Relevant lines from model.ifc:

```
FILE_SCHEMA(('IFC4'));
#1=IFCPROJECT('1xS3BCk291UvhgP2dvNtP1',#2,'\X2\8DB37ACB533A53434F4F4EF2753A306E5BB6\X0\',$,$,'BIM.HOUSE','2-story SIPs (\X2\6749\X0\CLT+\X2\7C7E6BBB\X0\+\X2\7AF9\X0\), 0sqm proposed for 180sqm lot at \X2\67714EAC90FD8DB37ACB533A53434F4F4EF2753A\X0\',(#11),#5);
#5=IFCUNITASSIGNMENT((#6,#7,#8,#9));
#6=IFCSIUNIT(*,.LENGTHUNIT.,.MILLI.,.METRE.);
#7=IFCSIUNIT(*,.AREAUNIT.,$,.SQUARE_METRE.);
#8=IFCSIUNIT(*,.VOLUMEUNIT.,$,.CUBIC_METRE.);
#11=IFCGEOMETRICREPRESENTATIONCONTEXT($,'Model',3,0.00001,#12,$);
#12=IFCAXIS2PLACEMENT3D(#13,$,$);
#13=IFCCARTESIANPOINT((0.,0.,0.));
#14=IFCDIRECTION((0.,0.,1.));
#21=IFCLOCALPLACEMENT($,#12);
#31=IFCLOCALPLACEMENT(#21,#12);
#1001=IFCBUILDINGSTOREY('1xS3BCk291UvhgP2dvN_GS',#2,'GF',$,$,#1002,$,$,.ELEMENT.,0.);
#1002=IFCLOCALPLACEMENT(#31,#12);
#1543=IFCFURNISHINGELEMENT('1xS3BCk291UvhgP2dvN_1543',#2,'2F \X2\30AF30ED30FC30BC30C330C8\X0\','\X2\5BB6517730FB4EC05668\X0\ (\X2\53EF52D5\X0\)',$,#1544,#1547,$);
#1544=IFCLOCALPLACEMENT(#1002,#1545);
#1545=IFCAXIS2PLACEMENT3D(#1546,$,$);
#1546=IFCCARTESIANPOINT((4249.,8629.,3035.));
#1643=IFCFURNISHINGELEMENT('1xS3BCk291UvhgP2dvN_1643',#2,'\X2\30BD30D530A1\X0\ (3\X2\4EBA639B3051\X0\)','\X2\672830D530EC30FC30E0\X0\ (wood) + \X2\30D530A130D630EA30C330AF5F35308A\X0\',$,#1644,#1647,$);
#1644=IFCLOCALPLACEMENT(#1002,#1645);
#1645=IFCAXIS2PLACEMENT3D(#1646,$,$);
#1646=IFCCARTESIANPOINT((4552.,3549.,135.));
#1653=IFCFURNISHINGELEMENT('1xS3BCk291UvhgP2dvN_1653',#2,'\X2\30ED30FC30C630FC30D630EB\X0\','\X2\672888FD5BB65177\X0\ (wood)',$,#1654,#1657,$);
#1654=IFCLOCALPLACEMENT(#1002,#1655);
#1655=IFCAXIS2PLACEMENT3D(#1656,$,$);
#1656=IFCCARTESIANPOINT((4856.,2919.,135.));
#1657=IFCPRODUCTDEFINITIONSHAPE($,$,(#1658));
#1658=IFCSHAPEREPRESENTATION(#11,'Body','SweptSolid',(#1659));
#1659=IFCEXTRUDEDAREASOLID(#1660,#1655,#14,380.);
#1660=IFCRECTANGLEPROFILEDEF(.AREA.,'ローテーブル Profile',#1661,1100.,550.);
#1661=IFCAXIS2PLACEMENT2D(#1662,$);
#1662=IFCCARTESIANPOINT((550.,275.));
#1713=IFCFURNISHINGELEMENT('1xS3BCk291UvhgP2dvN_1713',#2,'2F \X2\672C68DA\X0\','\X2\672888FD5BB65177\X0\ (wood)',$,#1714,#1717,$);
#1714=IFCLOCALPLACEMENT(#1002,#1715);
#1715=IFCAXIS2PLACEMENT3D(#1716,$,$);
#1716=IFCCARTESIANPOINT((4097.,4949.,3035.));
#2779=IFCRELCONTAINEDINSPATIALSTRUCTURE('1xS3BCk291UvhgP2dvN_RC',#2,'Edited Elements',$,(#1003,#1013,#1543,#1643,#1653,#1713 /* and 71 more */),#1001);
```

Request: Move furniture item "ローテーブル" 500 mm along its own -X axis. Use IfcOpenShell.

```python
import ifcopenshell
import ifcopenshell.api.geometry
import ifcopenshell.util.placement

model = ifcopenshell.open("model.ifc")

item = model.by_guid("1xS3BCk291UvhgP2dvN_1653")
matrix = ifcopenshell.util.placement.get_local_placement(item.ObjectPlacement)
matrix[:3, 3] -= matrix[:3, 0] * 500.0
ifcopenshell.api.geometry.edit_object_placement(model, product=item, matrix=matrix, is_si=False)

print(ifcopenshell.util.placement.get_local_placement(item.ObjectPlacement).round(3) + 0.0)

model.write("model_rev.ifc")
```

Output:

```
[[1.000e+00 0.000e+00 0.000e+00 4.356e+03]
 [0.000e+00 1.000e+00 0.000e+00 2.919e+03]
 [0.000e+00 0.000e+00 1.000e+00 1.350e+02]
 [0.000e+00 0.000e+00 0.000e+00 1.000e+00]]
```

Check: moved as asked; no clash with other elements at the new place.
